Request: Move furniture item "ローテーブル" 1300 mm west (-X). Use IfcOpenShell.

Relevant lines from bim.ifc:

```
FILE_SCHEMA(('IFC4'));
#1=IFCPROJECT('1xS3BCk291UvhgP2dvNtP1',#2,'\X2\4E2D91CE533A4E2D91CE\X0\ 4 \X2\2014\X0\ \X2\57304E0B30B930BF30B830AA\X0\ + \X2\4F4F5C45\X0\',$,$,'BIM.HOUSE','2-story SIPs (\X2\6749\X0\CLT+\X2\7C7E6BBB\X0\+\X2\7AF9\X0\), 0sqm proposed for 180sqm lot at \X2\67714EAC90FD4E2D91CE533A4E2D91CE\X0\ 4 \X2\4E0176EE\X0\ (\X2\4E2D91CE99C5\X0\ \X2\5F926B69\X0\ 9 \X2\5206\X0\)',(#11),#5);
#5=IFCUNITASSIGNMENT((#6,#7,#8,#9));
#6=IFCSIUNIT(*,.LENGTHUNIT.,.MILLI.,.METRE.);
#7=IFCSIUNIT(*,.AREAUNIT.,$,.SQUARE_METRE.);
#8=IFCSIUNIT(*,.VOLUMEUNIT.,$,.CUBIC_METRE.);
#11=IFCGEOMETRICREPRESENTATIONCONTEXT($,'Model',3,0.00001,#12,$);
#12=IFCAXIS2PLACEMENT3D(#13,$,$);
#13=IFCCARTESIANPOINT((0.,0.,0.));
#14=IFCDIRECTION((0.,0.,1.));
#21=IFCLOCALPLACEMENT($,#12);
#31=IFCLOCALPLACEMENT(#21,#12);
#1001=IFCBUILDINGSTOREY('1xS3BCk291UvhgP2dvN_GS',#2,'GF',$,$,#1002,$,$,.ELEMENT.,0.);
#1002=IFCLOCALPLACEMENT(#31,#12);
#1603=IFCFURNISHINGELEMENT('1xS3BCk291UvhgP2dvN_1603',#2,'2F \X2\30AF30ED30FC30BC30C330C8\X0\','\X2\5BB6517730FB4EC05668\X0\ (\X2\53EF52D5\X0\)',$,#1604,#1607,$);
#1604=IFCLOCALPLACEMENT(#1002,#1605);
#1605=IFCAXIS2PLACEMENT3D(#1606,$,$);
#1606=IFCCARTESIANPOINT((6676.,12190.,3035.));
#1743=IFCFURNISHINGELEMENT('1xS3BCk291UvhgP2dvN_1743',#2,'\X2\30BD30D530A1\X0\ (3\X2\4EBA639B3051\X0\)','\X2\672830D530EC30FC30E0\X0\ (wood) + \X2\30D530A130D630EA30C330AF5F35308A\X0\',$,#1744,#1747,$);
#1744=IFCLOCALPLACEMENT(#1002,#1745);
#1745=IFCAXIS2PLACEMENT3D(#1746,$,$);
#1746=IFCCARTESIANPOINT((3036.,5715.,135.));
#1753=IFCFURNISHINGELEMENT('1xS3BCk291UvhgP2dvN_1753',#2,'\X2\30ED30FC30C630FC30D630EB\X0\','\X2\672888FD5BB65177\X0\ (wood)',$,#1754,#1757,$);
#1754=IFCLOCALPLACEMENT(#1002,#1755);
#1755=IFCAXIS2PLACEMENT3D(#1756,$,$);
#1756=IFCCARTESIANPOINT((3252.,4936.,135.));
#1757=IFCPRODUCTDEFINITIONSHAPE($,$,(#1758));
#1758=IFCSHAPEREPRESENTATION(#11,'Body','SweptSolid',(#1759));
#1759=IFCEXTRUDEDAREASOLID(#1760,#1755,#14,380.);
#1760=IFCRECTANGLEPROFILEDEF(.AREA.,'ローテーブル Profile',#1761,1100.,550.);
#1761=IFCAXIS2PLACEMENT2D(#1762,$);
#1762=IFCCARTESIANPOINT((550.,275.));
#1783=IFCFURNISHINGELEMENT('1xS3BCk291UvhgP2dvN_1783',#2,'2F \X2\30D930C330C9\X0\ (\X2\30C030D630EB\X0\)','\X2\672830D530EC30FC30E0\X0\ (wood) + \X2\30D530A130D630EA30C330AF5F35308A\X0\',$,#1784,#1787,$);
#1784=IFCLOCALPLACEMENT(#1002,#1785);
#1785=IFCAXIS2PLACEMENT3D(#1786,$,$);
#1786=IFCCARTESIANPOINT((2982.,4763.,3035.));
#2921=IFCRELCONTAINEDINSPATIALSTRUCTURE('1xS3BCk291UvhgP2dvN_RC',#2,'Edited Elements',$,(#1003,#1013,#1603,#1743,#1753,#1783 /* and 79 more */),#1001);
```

```python
import ifcopenshell
import ifcopenshell.api.geometry
import ifcopenshell.util.placement
import ifcopenshell.util.unit

model = ifcopenshell.open("bim.ifc")
unit_scale = ifcopenshell.util.unit.calculate_unit_scale(model)

item = model.by_guid("1xS3BCk291UvhgP2dvN_1753")
matrix = ifcopenshell.util.placement.get_local_placement(item.ObjectPlacement)
matrix[0, 3] -= 1.3 / unit_scale
ifcopenshell.api.geometry.edit_object_placement(model, product=item, matrix=matrix, is_si=False)

print(ifcopenshell.util.placement.get_local_placement(item.ObjectPlacement).round(3) + 0.0)

model.write("bim_v2.ifc")
```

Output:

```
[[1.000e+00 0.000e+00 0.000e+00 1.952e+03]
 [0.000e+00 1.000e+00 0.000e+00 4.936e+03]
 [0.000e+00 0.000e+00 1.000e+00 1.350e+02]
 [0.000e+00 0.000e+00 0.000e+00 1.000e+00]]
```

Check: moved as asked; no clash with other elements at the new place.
